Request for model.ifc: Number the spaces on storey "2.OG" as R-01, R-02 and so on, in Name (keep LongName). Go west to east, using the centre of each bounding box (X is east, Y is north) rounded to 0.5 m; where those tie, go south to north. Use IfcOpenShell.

First a look at what the model holds.

```python
import ifcopenshell
import ifcopenshell.util.element
import ifcopenshell.util.placement

model = ifcopenshell.open("model.ifc")
print(model.schema)
storey = next(s for s in model.by_type("IfcBuildingStorey") if s.Name == "2.OG")
spaces = [e for e in ifcopenshell.util.element.get_decomposition(storey) if e.is_a("IfcSpace")]
for e in sorted(spaces, key=lambda e: e.id()):
    origin = ifcopenshell.util.placement.get_local_placement(e.ObjectPlacement)[:3, 3]
    print(e.id(), e.Name, e.LongName, origin.round(2) + 0.0, sep=" | ")
```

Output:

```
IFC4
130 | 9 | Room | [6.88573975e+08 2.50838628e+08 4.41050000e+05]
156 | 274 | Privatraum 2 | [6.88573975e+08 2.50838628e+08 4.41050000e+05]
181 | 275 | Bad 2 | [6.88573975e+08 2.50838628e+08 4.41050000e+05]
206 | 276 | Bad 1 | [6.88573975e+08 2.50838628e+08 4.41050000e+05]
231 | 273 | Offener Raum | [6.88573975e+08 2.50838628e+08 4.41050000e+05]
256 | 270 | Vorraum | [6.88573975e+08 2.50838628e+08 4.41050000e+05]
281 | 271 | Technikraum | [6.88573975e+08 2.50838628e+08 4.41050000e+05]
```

```python
import ifcopenshell
import ifcopenshell.geom
import ifcopenshell.util.element
import ifcopenshell.util.shape

model = ifcopenshell.open("model.ifc")
settings = ifcopenshell.geom.settings()
settings.set("use-world-coords", True)


def centre(element):
    shape = ifcopenshell.geom.create_shape(settings, element)
    return ifcopenshell.util.shape.get_bbox_centroid(shape.geometry)


storey = next(s for s in model.by_type("IfcBuildingStorey") if s.Name == "2.OG")
spaces = [e for e in ifcopenshell.util.element.get_decomposition(storey) if e.is_a("IfcSpace")]

# Insertion points can sit at a corner or the storey origin, so sort by the geometry (in metres).
centres = {e: centre(e) for e in spaces}
spaces.sort(key=lambda e: (round(centres[e][0] / 0.5), centres[e][1]))

for i, e in enumerate(spaces, start=1):
    number = f"R-{i:02d}"
    e.Name = number
    print(e.id(), number)

model.write("model_rev.ifc")
```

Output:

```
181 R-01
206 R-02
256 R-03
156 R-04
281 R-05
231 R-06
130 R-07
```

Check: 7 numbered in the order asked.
